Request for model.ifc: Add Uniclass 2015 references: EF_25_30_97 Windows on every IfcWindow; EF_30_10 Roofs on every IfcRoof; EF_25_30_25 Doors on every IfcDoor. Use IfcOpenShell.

First a look at what the model holds.

```python
import ifcopenshell

model = ifcopenshell.open("model.ifc")
print(model.schema)
print("classifications:", [c.Name for c in model.by_type("IfcClassification")])
for ifc_class in ("IfcDoor", "IfcRoof", "IfcStair", "IfcWall", "IfcWindow"):
    print(ifc_class, len(model.by_type(ifc_class)))
```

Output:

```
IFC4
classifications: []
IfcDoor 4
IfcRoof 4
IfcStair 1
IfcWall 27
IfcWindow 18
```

```python
import ifcopenshell
import ifcopenshell.api.classification

model = ifcopenshell.open("model.ifc")

system = ifcopenshell.api.classification.add_classification(model, classification="Uniclass 2015")

codes = {
    "IfcWindow": ("EF_25_30_97", "Windows"),
    "IfcRoof": ("EF_30_10", "Roofs"),
    "IfcDoor": ("EF_25_30_25", "Doors"),
}
for ifc_class, (code, name) in codes.items():
    products = model.by_type(ifc_class)
    ifcopenshell.api.classification.add_reference(
        model, products=products, classification=system, identification=code, name=name
    )
    print(code, len(products))

model.write("model_v2.ifc")
```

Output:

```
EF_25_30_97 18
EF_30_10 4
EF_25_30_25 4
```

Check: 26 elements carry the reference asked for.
